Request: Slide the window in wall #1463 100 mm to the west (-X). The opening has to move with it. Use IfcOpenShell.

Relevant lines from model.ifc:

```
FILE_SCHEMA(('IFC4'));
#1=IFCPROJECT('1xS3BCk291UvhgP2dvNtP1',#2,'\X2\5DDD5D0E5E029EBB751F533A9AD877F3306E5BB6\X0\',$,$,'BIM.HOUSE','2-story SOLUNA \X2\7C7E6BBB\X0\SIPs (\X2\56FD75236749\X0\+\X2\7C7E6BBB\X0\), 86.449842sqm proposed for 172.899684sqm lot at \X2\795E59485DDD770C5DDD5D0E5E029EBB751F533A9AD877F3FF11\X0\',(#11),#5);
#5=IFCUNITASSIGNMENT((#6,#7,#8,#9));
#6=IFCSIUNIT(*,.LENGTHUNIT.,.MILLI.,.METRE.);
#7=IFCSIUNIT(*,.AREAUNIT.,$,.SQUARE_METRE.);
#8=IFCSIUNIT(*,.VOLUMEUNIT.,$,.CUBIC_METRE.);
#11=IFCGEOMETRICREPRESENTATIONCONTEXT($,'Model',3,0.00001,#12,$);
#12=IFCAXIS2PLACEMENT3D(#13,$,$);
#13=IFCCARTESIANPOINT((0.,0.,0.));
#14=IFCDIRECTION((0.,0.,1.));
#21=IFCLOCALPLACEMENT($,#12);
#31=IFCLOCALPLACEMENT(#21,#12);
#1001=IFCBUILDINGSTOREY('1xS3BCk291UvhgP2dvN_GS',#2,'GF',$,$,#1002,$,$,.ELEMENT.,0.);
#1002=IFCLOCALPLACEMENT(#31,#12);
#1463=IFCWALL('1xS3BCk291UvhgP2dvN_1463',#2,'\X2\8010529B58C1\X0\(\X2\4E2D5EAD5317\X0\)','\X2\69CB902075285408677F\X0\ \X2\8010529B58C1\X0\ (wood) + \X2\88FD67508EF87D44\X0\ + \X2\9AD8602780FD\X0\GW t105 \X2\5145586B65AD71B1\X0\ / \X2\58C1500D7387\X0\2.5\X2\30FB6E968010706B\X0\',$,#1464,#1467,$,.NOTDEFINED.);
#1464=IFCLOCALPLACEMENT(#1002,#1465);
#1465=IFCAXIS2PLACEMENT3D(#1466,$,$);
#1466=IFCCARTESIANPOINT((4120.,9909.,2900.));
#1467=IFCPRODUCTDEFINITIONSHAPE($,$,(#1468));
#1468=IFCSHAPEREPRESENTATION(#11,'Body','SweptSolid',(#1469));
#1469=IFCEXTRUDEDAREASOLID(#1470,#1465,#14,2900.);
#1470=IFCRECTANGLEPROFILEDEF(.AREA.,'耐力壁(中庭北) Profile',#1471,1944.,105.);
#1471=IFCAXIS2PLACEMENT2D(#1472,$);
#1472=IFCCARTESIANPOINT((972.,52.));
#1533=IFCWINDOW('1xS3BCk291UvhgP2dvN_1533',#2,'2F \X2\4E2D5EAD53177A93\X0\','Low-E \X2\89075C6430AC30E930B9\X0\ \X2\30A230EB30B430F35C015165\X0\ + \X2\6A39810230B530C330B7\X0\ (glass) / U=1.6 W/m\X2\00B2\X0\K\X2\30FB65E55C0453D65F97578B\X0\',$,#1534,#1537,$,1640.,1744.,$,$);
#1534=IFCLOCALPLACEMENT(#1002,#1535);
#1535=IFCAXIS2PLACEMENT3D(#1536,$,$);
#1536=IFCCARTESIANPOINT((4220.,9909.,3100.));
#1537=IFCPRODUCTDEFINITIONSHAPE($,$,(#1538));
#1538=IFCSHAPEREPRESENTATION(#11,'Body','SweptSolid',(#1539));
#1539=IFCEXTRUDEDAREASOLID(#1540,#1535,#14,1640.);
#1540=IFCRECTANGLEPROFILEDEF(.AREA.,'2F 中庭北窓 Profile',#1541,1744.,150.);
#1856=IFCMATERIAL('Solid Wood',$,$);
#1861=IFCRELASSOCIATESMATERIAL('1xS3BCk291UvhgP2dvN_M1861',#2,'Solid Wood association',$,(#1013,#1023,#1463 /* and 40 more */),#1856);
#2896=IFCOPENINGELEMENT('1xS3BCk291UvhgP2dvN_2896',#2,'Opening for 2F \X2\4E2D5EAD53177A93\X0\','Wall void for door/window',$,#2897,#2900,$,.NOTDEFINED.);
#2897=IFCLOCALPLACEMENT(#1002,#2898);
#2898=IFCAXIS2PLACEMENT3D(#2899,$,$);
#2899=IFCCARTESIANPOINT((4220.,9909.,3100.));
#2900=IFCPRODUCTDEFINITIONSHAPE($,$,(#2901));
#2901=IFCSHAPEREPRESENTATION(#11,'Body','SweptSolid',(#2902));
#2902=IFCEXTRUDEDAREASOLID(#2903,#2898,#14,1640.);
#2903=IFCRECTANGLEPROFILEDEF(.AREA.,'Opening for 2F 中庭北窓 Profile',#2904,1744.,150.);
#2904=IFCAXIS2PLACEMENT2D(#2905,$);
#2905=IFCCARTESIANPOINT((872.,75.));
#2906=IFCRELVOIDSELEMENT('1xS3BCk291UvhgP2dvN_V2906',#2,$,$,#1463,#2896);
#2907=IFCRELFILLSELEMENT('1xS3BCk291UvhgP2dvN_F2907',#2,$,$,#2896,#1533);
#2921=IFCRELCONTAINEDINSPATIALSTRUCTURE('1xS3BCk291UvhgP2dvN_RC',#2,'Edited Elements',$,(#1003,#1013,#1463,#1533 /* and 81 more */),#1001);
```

```python
import ifcopenshell
import ifcopenshell.api.geometry
import ifcopenshell.util.placement
import ifcopenshell.util.unit

model = ifcopenshell.open("model.ifc")
unit_scale = ifcopenshell.util.unit.calculate_unit_scale(model)

window = model.by_guid("1xS3BCk291UvhgP2dvN_1533")
opening = window.FillsVoids[0].RelatingOpeningElement
wall = opening.VoidsElements[0].RelatingBuildingElement

wall_matrix = ifcopenshell.util.placement.get_local_placement(wall.ObjectPlacement)
shift = wall_matrix[:3, 0] * -0.1 / unit_scale
before = ifcopenshell.util.placement.get_local_placement(window.ObjectPlacement)[:3, 3].copy()

# The window is not placed relative to its opening, so move both.
for product in (opening, window):
    matrix = ifcopenshell.util.placement.get_local_placement(product.ObjectPlacement)
    matrix[:3, 3] += shift
    ifcopenshell.api.geometry.edit_object_placement(model, product=product, matrix=matrix, is_si=False)

after = ifcopenshell.util.placement.get_local_placement(window.ObjectPlacement)[:3, 3]
print("window moved by", (after - before).round(3) + 0.0)

model.write("model_rev.ifc")
```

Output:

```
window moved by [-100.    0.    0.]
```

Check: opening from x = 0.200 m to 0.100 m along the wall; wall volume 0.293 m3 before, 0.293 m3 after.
